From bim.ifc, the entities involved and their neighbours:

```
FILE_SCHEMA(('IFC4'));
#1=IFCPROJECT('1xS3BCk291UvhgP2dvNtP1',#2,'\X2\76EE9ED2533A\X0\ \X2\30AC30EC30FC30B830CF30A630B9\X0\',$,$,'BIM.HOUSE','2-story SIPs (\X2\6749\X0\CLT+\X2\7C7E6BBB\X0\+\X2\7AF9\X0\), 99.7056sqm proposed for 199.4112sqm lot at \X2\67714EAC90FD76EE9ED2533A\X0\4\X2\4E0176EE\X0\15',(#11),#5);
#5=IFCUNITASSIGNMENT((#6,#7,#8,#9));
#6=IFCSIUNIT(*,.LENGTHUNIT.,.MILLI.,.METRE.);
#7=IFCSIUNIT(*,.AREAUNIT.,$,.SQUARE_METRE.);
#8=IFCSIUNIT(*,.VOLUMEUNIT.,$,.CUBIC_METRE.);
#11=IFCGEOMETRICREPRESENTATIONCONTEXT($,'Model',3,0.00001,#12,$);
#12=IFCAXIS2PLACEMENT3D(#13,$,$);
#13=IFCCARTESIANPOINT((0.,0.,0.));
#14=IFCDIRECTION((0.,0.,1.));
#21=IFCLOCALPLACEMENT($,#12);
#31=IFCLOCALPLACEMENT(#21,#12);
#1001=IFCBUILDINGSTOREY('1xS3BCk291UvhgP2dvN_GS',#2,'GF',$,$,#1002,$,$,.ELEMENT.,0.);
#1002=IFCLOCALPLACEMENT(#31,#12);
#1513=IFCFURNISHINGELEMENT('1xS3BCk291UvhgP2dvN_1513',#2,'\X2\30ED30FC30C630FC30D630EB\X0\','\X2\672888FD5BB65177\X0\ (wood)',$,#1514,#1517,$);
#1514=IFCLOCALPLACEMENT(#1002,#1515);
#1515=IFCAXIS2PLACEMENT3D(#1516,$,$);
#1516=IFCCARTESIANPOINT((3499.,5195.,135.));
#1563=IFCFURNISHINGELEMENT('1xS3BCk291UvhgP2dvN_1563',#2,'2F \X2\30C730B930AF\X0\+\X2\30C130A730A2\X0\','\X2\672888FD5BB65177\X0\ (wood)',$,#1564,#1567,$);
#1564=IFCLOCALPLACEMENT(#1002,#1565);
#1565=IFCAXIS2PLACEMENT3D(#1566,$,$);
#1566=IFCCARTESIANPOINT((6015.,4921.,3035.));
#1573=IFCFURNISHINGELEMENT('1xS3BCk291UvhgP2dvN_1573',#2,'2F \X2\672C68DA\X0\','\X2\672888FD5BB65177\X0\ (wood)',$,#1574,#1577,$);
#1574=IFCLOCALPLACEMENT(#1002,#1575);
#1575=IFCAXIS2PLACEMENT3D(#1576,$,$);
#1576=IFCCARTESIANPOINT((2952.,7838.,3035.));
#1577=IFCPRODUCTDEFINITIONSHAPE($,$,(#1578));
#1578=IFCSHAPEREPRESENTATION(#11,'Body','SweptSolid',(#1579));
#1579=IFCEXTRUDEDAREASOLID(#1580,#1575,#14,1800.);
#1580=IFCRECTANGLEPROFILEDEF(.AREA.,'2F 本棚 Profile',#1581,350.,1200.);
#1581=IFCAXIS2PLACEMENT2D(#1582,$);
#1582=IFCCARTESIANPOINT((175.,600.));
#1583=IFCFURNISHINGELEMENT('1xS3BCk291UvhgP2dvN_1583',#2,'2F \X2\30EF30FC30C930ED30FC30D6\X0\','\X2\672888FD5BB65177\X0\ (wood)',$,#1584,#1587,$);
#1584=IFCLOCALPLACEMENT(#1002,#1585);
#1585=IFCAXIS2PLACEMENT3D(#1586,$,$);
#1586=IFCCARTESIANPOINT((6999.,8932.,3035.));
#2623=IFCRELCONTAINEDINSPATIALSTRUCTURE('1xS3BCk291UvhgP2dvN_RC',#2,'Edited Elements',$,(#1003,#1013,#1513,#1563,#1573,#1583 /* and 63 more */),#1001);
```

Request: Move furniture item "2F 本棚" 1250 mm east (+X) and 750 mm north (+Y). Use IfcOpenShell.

```python
import ifcopenshell
import ifcopenshell.api.geometry
import ifcopenshell.util.placement
import ifcopenshell.util.unit

model = ifcopenshell.open("bim.ifc")
unit_scale = ifcopenshell.util.unit.calculate_unit_scale(model)

item = model.by_guid("1xS3BCk291UvhgP2dvN_1573")
matrix = ifcopenshell.util.placement.get_local_placement(item.ObjectPlacement)
matrix[0, 3] += 1.25 / unit_scale
matrix[1, 3] += 0.75 / unit_scale
ifcopenshell.api.geometry.edit_object_placement(model, product=item, matrix=matrix, is_si=False)

print(ifcopenshell.util.placement.get_local_placement(item.ObjectPlacement).round(3) + 0.0)

model.write("bim_v2.ifc")
```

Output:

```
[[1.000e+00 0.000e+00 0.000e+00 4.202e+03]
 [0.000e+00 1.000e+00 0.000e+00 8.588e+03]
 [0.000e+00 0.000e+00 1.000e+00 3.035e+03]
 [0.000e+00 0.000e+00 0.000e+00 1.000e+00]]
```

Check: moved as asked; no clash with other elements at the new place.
